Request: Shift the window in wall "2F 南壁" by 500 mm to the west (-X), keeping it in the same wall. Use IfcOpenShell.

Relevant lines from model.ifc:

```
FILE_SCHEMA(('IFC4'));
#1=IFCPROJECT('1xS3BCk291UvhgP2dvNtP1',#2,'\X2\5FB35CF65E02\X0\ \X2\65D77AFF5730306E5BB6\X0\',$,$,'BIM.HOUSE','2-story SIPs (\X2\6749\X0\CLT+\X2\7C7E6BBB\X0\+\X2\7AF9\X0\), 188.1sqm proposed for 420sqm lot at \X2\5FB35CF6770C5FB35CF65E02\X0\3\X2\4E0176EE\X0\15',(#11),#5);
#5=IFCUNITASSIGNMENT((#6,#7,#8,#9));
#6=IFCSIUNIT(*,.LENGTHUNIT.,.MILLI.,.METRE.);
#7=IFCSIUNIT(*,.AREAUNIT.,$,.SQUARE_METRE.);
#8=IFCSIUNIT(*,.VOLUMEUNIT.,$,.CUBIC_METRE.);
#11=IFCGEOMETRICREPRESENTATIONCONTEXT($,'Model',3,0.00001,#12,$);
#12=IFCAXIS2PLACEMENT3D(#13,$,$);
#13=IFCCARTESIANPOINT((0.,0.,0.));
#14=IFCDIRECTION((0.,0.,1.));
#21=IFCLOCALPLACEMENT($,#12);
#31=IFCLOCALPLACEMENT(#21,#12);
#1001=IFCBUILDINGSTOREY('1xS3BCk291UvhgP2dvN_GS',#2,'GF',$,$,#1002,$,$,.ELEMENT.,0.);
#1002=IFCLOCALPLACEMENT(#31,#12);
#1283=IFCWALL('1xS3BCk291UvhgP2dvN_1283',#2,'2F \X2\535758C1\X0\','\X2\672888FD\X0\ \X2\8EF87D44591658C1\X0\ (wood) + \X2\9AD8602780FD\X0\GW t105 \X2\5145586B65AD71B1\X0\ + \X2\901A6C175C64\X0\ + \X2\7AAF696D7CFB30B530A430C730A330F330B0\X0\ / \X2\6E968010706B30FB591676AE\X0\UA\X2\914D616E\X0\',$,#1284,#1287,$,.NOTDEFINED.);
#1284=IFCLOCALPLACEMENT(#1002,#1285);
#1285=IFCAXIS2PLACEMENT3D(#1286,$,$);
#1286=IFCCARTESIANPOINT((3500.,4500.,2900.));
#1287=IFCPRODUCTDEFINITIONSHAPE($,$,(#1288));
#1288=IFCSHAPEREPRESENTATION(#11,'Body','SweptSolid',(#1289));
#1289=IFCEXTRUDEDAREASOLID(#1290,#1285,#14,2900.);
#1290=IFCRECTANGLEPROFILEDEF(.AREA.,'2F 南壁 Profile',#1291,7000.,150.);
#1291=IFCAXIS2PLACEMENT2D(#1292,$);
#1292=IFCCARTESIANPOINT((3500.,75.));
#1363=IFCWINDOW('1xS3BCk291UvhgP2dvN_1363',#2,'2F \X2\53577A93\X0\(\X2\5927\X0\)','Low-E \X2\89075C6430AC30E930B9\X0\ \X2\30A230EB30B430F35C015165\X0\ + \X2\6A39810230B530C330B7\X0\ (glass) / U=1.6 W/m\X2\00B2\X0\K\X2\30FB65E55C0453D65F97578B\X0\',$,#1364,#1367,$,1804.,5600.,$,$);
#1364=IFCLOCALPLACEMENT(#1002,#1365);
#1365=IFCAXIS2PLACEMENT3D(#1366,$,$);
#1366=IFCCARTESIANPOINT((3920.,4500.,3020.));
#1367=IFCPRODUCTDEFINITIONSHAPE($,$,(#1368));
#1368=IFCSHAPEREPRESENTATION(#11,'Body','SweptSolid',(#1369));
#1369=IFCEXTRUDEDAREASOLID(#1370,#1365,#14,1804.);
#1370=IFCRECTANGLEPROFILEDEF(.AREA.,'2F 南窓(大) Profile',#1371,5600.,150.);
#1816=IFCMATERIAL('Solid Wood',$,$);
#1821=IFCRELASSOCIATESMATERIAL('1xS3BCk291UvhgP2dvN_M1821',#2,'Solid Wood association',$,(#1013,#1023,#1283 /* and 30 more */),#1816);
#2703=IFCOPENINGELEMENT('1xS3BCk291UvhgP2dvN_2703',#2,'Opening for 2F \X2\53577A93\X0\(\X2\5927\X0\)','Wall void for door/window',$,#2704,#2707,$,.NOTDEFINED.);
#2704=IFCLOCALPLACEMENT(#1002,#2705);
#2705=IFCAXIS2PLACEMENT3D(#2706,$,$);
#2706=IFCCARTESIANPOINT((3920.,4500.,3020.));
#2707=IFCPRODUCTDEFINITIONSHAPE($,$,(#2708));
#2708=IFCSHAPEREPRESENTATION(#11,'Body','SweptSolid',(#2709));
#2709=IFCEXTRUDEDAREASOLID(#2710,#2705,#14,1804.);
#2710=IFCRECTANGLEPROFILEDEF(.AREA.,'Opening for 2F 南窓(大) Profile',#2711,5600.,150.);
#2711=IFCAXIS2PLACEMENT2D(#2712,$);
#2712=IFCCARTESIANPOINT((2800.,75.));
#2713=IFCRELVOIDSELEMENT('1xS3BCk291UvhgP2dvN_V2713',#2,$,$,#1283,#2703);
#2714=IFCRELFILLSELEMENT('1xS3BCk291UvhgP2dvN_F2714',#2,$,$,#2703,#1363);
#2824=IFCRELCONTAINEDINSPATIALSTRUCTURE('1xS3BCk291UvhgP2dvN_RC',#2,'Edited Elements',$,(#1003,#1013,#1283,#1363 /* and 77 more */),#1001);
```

```python
import ifcopenshell
import ifcopenshell.api.geometry
import ifcopenshell.util.placement

model = ifcopenshell.open("model.ifc")

window = model.by_guid("1xS3BCk291UvhgP2dvN_1363")
opening = window.FillsVoids[0].RelatingOpeningElement
wall = opening.VoidsElements[0].RelatingBuildingElement

wall_matrix = ifcopenshell.util.placement.get_local_placement(wall.ObjectPlacement)
shift = wall_matrix[:3, 0] * -500.0
before = ifcopenshell.util.placement.get_local_placement(window.ObjectPlacement)[:3, 3].copy()

# The window is not placed relative to its opening, so move both.
for product in (opening, window):
    matrix = ifcopenshell.util.placement.get_local_placement(product.ObjectPlacement)
    matrix[:3, 3] += shift
    ifcopenshell.api.geometry.edit_object_placement(model, product=product, matrix=matrix, is_si=False)

after = ifcopenshell.util.placement.get_local_placement(window.ObjectPlacement)[:3, 3]
print("window moved by", (after - before).round(3) + 0.0)

model.write("model_v2.ifc")
```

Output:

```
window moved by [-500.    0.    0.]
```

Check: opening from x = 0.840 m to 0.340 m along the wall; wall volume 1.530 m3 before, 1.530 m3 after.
